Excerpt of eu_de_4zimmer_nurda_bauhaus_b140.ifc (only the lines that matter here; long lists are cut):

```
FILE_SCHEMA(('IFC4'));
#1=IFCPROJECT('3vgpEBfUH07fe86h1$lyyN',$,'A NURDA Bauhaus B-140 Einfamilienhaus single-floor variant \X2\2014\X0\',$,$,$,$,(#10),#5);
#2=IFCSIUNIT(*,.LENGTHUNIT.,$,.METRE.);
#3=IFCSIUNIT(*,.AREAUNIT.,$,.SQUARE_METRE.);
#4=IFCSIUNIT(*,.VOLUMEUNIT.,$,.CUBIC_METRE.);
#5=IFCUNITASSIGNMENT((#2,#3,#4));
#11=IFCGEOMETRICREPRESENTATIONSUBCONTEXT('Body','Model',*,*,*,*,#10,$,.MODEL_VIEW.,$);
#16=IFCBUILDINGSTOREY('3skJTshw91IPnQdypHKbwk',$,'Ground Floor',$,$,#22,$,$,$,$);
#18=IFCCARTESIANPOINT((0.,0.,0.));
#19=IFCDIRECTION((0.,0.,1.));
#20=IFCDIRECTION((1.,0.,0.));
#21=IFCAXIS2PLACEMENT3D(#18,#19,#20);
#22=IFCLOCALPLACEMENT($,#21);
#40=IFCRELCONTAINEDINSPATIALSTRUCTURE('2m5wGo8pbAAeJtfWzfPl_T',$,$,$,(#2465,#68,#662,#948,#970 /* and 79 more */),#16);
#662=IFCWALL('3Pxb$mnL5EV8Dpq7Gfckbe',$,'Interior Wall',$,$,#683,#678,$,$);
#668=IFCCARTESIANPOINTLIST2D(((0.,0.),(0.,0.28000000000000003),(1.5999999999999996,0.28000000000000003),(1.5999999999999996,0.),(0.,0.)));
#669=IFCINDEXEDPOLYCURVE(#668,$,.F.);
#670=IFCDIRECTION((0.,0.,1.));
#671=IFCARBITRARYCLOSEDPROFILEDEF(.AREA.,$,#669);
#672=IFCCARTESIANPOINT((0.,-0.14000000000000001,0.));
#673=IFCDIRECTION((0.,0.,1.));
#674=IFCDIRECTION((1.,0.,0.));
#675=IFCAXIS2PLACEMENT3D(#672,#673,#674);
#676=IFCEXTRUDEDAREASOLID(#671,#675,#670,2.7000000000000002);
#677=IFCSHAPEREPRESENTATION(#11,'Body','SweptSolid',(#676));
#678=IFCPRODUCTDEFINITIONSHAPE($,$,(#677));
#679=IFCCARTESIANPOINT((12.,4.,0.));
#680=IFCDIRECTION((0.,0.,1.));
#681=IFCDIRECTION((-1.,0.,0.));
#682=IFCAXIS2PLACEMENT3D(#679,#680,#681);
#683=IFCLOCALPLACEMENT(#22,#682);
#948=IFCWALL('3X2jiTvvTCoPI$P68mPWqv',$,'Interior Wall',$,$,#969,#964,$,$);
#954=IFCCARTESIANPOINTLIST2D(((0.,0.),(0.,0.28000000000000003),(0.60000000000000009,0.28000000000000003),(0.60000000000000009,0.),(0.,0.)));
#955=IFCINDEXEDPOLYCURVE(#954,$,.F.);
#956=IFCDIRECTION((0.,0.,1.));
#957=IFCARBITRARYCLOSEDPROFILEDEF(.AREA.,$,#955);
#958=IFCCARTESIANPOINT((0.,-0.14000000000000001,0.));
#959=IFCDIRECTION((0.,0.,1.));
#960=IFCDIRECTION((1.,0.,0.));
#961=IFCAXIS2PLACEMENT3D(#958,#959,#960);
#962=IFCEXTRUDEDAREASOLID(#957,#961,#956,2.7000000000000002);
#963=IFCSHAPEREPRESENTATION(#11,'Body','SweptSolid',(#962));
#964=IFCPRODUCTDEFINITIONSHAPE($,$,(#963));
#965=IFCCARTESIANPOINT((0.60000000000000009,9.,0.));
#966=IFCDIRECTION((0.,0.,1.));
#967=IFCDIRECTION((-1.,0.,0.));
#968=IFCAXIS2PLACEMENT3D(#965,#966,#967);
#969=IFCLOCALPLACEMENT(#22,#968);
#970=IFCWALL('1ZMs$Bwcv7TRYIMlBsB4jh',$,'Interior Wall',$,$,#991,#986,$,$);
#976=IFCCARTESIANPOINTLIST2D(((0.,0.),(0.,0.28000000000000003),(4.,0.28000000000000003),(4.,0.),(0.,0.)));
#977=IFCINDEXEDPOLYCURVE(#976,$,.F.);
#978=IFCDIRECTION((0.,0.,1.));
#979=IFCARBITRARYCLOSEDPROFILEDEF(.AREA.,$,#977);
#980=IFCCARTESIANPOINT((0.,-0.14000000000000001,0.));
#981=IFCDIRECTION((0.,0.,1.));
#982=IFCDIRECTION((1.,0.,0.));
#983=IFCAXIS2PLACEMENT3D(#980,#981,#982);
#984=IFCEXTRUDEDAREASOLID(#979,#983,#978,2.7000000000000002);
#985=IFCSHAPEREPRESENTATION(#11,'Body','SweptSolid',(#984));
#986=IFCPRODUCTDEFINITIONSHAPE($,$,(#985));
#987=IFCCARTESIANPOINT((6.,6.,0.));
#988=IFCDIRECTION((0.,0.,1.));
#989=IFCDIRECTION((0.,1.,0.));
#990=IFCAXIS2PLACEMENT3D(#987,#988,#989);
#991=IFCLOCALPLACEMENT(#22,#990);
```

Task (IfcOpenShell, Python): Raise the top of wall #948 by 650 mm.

```python
import ifcopenshell
import ifcopenshell.geom
import ifcopenshell.util.representation
import ifcopenshell.util.shape
import ifcopenshell.util.unit

model = ifcopenshell.open("eu_de_4zimmer_nurda_bauhaus_b140.ifc")
unit_scale = ifcopenshell.util.unit.calculate_unit_scale(model)
settings = ifcopenshell.geom.settings()


def volume(element):
    """Net volume in cubic metres, openings subtracted."""
    shape = ifcopenshell.geom.create_shape(settings, element)
    return ifcopenshell.util.shape.get_volume(shape.geometry)


wall = model.by_id(948)
before = volume(wall)

body = ifcopenshell.util.representation.get_representation(wall, "Model", "Body")
solid = body.Items[0]
old_height = solid.Depth
solid.Depth += 0.65 / unit_scale
after = volume(wall)

print(f"height {old_height:g} -> {solid.Depth:g}, volume {before:.3f} -> {after:.3f} m3")

model.write("eu_de_4zimmer_nurda_bauhaus_b140_v2.ifc")
```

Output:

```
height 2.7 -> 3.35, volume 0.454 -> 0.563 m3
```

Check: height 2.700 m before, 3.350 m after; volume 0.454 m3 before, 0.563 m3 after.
